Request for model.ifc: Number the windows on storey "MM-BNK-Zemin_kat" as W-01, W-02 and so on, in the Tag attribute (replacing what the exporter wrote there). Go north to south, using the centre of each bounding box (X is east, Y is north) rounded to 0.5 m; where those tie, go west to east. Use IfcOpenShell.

First a look at what the model holds.

```python
import ifcopenshell
import ifcopenshell.util.element
import ifcopenshell.util.placement

model = ifcopenshell.open("model.ifc")
print(model.schema)
storey = next(s for s in model.by_type("IfcBuildingStorey") if s.Name == "MM-BNK-Zemin_kat")
windows = [e for e in ifcopenshell.util.element.get_decomposition(storey) if e.is_a("IfcWindow")]
for e in sorted(windows, key=lambda e: e.id()):
    origin = ifcopenshell.util.placement.get_local_placement(e.ObjectPlacement)[:3, 3]
    print(e.id(), e.Tag, e.Name, origin.round(2) + 0.0, sep=" | ")
```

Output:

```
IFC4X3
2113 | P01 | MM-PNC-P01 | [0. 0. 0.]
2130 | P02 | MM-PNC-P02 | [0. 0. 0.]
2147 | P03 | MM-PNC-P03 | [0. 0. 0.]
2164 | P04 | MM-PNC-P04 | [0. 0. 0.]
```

```python
import ifcopenshell
import ifcopenshell.geom
import ifcopenshell.util.element
import ifcopenshell.util.shape

model = ifcopenshell.open("model.ifc")
settings = ifcopenshell.geom.settings()
settings.set("use-world-coords", True)


def centre(element):
    shape = ifcopenshell.geom.create_shape(settings, element)
    return ifcopenshell.util.shape.get_bbox_centroid(shape.geometry)


storey = next(s for s in model.by_type("IfcBuildingStorey") if s.Name == "MM-BNK-Zemin_kat")
windows = [e for e in ifcopenshell.util.element.get_decomposition(storey) if e.is_a("IfcWindow")]

# Insertion points can sit at a corner or the storey origin, so sort by the geometry (in metres).
centres = {e: centre(e) for e in windows}
windows.sort(key=lambda e: (-round(centres[e][1] / 0.5), centres[e][0]))

for i, e in enumerate(windows, start=1):
    number = f"W-{i:02d}"
    e.Tag = number
    print(e.id(), number)

model.write("model-out.ifc")
```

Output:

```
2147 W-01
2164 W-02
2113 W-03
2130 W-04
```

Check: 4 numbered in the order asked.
